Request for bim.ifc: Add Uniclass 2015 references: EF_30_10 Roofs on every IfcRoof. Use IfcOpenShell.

First a look at what the model holds.

```python
import ifcopenshell

model = ifcopenshell.open("bim.ifc")
print(model.schema)
print("classifications:", [c.Name for c in model.by_type("IfcClassification")])
for ifc_class in ("IfcDoor", "IfcRoof", "IfcStair", "IfcWall", "IfcWindow"):
    print(ifc_class, len(model.by_type(ifc_class)))
```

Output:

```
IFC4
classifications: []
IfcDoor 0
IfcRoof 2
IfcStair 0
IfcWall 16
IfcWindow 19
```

```python
import ifcopenshell
import ifcopenshell.api.classification

model = ifcopenshell.open("bim.ifc")

system = ifcopenshell.api.classification.add_classification(model, classification="Uniclass 2015")

codes = {
    "IfcRoof": ("EF_30_10", "Roofs"),
}
for ifc_class, (code, name) in codes.items():
    products = model.by_type(ifc_class)
    ifcopenshell.api.classification.add_reference(
        model, products=products, classification=system, identification=code, name=name
    )
    print(code, len(products))

model.write("bim_edited.ifc")
```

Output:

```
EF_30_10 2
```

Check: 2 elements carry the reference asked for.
